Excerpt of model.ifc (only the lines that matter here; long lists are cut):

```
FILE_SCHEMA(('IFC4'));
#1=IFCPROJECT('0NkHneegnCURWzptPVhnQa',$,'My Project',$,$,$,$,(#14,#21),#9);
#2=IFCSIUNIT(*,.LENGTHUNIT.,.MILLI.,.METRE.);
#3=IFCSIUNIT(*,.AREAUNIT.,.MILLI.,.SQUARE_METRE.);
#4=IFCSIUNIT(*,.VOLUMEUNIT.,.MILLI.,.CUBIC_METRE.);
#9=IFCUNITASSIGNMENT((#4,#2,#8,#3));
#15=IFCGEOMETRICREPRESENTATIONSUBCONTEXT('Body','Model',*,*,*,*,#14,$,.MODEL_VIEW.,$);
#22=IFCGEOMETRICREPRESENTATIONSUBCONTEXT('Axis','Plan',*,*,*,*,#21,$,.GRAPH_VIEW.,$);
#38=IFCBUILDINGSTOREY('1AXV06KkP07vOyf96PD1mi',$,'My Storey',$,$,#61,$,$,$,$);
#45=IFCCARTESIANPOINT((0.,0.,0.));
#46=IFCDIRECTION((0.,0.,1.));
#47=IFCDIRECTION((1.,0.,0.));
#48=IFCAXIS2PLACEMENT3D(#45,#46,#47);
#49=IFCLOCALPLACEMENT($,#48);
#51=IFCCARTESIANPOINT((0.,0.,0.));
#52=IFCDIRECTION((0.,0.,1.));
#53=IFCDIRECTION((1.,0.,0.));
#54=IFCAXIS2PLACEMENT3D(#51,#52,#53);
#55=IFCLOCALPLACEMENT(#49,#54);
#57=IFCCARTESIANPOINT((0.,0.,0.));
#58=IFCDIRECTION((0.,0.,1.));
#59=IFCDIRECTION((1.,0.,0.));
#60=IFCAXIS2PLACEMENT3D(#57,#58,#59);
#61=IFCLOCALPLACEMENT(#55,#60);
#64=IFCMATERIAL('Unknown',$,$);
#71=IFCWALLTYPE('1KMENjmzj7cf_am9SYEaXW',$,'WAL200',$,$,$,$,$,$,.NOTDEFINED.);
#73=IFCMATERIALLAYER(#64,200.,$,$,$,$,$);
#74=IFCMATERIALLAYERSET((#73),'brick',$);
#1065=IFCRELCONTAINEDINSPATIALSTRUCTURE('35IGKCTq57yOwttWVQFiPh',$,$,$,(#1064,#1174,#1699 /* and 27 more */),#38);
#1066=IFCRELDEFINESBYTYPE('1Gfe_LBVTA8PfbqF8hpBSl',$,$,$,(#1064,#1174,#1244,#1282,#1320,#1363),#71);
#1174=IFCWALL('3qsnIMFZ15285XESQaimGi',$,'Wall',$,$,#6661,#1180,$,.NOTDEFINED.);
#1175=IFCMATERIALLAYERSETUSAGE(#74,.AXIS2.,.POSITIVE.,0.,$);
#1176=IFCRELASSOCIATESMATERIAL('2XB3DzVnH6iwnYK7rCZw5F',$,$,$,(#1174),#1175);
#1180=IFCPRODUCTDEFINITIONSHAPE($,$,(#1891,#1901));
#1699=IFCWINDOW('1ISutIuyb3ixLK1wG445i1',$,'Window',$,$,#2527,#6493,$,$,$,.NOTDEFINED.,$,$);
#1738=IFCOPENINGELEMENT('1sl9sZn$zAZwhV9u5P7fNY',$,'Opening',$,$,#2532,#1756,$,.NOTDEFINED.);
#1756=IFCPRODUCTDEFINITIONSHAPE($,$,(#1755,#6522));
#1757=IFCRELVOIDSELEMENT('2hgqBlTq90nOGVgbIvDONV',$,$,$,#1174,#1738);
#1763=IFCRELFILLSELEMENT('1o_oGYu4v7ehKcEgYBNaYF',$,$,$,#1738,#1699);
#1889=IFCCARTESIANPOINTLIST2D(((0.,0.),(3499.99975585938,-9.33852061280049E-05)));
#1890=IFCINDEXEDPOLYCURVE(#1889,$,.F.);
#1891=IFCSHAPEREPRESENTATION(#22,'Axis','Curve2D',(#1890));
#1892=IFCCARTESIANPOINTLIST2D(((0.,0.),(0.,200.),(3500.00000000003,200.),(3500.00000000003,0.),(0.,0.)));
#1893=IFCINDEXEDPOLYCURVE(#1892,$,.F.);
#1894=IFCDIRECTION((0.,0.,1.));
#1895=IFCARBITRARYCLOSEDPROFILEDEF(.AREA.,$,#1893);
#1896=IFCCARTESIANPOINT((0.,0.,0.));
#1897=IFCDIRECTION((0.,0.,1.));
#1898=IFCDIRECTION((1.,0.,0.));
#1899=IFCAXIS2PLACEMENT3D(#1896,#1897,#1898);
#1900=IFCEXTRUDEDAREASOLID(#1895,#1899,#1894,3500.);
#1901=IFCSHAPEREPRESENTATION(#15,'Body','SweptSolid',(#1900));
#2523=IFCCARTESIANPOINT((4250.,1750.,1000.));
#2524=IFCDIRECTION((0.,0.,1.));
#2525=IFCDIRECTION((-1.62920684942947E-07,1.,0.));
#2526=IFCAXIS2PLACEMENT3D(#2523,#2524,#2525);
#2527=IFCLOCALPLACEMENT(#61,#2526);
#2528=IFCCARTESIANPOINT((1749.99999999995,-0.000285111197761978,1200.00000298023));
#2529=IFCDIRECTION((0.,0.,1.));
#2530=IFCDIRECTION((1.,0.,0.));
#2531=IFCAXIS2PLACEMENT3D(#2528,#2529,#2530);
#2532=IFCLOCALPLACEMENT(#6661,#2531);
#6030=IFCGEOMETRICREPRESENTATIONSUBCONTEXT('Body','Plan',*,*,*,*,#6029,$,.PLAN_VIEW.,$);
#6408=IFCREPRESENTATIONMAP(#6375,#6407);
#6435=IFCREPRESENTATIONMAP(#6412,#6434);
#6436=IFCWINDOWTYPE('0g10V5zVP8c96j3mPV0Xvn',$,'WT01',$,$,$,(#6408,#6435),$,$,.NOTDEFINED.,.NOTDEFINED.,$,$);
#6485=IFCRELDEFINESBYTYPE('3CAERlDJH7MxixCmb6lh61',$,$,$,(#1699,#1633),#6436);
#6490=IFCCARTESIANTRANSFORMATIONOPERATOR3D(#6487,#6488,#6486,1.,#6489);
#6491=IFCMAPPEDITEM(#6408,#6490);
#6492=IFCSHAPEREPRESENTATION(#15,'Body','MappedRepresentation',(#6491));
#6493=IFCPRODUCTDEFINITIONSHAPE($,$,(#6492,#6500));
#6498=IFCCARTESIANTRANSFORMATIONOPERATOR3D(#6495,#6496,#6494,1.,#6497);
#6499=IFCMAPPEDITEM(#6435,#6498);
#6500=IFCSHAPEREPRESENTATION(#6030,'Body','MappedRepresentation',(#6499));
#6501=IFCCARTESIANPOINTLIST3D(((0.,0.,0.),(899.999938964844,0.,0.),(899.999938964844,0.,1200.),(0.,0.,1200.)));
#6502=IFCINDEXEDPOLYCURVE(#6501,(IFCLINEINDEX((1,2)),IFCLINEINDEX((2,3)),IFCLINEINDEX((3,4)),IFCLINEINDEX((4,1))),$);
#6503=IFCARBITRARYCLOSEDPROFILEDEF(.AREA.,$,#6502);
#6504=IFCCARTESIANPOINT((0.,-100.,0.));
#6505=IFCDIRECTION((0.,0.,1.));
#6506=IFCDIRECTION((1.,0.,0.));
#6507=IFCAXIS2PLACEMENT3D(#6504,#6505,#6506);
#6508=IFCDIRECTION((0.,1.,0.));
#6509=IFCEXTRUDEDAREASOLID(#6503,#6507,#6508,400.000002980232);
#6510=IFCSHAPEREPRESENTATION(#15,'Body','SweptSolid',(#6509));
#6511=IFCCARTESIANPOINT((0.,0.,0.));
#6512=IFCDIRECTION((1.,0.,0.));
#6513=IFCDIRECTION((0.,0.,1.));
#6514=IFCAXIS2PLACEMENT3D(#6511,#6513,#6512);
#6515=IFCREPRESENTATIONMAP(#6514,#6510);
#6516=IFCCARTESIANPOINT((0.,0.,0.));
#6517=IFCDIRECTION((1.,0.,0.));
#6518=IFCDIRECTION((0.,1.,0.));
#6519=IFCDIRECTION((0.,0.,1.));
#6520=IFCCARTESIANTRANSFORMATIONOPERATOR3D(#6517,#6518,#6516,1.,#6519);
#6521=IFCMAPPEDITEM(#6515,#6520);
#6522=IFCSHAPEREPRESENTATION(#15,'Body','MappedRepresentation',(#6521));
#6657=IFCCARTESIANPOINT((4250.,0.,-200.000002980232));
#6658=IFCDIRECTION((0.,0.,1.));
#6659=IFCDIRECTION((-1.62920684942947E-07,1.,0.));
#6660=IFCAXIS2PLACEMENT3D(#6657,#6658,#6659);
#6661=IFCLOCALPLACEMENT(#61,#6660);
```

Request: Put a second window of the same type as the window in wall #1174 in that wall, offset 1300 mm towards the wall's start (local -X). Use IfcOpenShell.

```python
import ifcopenshell
import ifcopenshell.api.feature
import ifcopenshell.api.geometry
import ifcopenshell.api.root
import ifcopenshell.geom
import ifcopenshell.util.element
import ifcopenshell.util.placement
import ifcopenshell.util.shape
import ifcopenshell.util.unit

model = ifcopenshell.open("model.ifc")
unit_scale = ifcopenshell.util.unit.calculate_unit_scale(model)
settings = ifcopenshell.geom.settings()


def volume(element):
    """Net volume in cubic metres, openings subtracted."""
    shape = ifcopenshell.geom.create_shape(settings, element)
    return ifcopenshell.util.shape.get_volume(shape.geometry)


window = model.by_id(1699)
opening = window.FillsVoids[0].RelatingOpeningElement
wall = opening.VoidsElements[0].RelatingBuildingElement
before = volume(wall)
shift = ifcopenshell.util.placement.get_local_placement(wall.ObjectPlacement)[:3, 0] * -1.3 / unit_scale

# copy_class copies the void relationship, type, container and properties, but no geometry.
new_opening = ifcopenshell.api.root.copy_class(model, product=opening)
new_opening.Representation = ifcopenshell.util.element.copy_deep(
    model, opening.Representation, exclude=["IfcGeometricRepresentationContext", "IfcRepresentationMap"]
)
new_window = ifcopenshell.api.root.copy_class(model, product=window)
new_window.Representation = ifcopenshell.util.element.copy_deep(
    model, window.Representation, exclude=["IfcGeometricRepresentationContext", "IfcRepresentationMap"]
)
ifcopenshell.api.feature.add_filling(model, opening=new_opening, element=new_window)

for old, new in ((opening, new_opening), (window, new_window)):
    matrix = ifcopenshell.util.placement.get_local_placement(old.ObjectPlacement)
    matrix[:3, 3] += shift
    ifcopenshell.api.geometry.edit_object_placement(model, product=new, matrix=matrix, is_si=False)

after = volume(wall)

print(f"wall volume {before:.3f} -> {after:.3f} m3")

model.write("model-out.ifc")
```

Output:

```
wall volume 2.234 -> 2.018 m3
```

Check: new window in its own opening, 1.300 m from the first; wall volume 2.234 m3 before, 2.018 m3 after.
